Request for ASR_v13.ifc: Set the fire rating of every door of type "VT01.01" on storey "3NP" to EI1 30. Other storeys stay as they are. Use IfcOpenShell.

First a look at what the model holds.

```python
import ifcopenshell
import ifcopenshell.util.element

model = ifcopenshell.open("ASR_v13.ifc")
print(model.schema)
storey = next(s for s in model.by_type("IfcBuildingStorey") if s.Name == "3NP")
doors = [e for e in ifcopenshell.util.element.get_decomposition(storey) if e.is_a("IfcDoor")]
seen = {}
for e in doors:
    element_type = ifcopenshell.util.element.get_type(e)
    key = (element_type.Name if element_type != e and element_type else None, ifcopenshell.util.element.get_pset(e, "Pset_DoorCommon", "FireRating"))
    seen[key] = seen.get(key, 0) + 1
for (name, value), count in sorted(seen.items(), key=str):
    print(count, "x", name, "|", value)
```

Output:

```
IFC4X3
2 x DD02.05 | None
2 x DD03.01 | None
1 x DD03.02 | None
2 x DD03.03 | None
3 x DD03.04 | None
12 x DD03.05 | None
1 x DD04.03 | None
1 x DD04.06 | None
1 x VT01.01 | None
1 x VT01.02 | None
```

```python
import ifcopenshell
import ifcopenshell.api.pset
import ifcopenshell.util.element

model = ifcopenshell.open("ASR_v13.ifc")

storey = next(s for s in model.by_type("IfcBuildingStorey") if s.Name == "3NP")
doors = [e for e in ifcopenshell.util.element.get_decomposition(storey) if e.is_a("IfcDoor")]

count = 0
for e in doors:
    element_type = ifcopenshell.util.element.get_type(e)
    if element_type in (None, e) or element_type.Name != "VT01.01":
        continue
    # add_pset returns the element's existing set when there is one.
    pset = ifcopenshell.api.pset.add_pset(model, product=e, name="Pset_DoorCommon")
    ifcopenshell.api.pset.edit_pset(model, pset=pset, properties={"FireRating": "EI1 30"})
    count += 1

print(count, "doors updated")

model.write("ASR_v13_updated.ifc")
```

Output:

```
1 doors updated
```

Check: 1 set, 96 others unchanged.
